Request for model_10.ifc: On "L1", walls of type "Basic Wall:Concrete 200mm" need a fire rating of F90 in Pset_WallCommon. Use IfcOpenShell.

First a look at what the model holds.

```python
import ifcopenshell
import ifcopenshell.util.element

model = ifcopenshell.open("model_10.ifc")
print(model.schema)
storey = next(s for s in model.by_type("IfcBuildingStorey") if s.Name == "L1")
walls = [e for e in ifcopenshell.util.element.get_decomposition(storey) if e.is_a("IfcWall")]
seen = {}
for e in walls:
    element_type = ifcopenshell.util.element.get_type(e)
    key = (element_type.Name if element_type != e and element_type else None, ifcopenshell.util.element.get_pset(e, "Pset_WallCommon", "FireRating"))
    seen[key] = seen.get(key, 0) + 1
for (name, value), count in sorted(seen.items(), key=str):
    print(count, "x", name, "|", value)
```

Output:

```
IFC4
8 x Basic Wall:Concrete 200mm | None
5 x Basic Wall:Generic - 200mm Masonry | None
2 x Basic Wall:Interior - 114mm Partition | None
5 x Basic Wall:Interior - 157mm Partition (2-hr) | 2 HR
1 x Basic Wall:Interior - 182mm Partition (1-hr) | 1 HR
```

```python
import ifcopenshell
import ifcopenshell.api.pset
import ifcopenshell.util.element

model = ifcopenshell.open("model_10.ifc")

storey = next(s for s in model.by_type("IfcBuildingStorey") if s.Name == "L1")
walls = [e for e in ifcopenshell.util.element.get_decomposition(storey) if e.is_a("IfcWall")]

count = 0
for e in walls:
    element_type = ifcopenshell.util.element.get_type(e)
    if element_type in (None, e) or element_type.Name != "Basic Wall:Concrete 200mm":
        continue
    # add_pset returns the element's existing set when there is one.
    pset = ifcopenshell.api.pset.add_pset(model, product=e, name="Pset_WallCommon")
    ifcopenshell.api.pset.edit_pset(model, pset=pset, properties={"FireRating": "F90"})
    count += 1

print(count, "walls updated")

model.write("model_10_edited.ifc")
```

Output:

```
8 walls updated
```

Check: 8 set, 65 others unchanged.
